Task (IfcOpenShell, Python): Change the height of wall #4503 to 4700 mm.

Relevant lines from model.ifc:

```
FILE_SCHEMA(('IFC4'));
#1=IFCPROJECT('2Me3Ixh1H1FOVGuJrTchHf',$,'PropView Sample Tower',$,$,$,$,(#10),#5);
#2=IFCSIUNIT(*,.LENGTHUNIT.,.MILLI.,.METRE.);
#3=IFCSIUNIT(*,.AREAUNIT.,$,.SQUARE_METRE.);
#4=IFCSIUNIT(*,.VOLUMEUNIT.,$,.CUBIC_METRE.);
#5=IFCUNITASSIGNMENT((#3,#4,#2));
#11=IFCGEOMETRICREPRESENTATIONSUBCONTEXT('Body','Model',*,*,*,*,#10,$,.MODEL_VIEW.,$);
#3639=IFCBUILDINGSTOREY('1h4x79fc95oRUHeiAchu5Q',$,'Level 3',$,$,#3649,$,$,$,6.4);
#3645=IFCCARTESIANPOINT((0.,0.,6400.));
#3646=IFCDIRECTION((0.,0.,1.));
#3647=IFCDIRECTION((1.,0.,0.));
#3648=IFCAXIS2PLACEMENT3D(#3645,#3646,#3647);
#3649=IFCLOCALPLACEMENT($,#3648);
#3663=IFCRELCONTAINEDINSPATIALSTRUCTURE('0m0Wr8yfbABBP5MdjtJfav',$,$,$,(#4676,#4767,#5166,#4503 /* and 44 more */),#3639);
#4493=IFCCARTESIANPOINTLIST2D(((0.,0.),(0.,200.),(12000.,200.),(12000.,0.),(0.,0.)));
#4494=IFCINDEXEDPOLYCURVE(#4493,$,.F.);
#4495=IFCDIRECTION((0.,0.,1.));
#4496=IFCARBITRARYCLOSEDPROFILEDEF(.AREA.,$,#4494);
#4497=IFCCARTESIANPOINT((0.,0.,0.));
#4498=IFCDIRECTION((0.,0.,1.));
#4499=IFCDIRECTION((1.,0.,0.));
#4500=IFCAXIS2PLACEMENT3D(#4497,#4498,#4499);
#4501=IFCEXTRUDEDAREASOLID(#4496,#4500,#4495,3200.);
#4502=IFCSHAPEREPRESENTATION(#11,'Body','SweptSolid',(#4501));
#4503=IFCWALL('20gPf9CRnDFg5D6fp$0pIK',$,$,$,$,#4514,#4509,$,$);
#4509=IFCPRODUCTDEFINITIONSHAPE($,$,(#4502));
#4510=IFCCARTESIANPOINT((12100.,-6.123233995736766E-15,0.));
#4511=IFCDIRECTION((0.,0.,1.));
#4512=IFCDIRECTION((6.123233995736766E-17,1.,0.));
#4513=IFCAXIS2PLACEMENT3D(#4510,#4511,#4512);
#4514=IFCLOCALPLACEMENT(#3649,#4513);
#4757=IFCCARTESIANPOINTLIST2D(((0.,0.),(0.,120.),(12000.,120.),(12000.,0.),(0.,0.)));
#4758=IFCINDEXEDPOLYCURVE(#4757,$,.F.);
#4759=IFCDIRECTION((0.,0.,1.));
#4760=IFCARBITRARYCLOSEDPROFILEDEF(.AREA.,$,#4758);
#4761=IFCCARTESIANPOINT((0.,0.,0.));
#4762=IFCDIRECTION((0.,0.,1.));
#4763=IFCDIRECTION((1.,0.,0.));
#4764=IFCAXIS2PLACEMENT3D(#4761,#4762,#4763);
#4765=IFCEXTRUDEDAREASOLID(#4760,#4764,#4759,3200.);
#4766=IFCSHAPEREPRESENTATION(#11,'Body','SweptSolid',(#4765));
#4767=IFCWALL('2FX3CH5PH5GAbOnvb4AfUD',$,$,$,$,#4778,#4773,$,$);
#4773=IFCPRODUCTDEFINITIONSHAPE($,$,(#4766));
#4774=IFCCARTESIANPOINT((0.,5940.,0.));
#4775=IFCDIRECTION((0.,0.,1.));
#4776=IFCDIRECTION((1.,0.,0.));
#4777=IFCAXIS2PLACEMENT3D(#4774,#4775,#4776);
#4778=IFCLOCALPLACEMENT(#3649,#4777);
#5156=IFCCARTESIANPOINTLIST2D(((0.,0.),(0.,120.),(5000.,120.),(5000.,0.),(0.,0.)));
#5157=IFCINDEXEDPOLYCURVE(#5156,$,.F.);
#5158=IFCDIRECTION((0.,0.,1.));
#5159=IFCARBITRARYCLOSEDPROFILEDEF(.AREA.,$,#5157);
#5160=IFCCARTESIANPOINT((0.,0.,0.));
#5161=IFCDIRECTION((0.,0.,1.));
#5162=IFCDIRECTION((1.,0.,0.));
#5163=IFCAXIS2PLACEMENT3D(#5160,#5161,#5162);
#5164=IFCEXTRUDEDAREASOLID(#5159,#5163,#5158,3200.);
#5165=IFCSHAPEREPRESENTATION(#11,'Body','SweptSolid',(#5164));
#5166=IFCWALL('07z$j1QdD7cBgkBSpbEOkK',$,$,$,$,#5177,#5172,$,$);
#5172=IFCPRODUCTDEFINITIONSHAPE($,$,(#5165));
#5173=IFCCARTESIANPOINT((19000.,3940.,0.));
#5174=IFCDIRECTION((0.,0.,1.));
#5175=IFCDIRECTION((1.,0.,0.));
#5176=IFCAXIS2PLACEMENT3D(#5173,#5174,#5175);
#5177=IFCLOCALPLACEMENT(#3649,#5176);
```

```python
import ifcopenshell
import ifcopenshell.geom
import ifcopenshell.util.representation
import ifcopenshell.util.shape

model = ifcopenshell.open("model.ifc")
settings = ifcopenshell.geom.settings()


def volume(element):
    """Net volume in cubic metres, openings subtracted."""
    shape = ifcopenshell.geom.create_shape(settings, element)
    return ifcopenshell.util.shape.get_volume(shape.geometry)


wall = model.by_guid("20gPf9CRnDFg5D6fp$0pIK")
before = volume(wall)

body = ifcopenshell.util.representation.get_representation(wall, "Model", "Body")
solid = body.Items[0]
old_height = solid.Depth
solid.Depth = 4700.0
after = volume(wall)

print(f"height {old_height:g} -> {solid.Depth:g}, volume {before:.3f} -> {after:.3f} m3")

model.write("model_v2.ifc")
```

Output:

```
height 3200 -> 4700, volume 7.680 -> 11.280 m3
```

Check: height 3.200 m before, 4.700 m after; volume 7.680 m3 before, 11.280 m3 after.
